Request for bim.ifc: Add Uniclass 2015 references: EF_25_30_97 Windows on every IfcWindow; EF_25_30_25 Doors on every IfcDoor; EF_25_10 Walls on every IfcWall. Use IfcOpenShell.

First a look at what the model holds.

```python
import ifcopenshell

model = ifcopenshell.open("bim.ifc")
print(model.schema)
print("classifications:", [c.Name for c in model.by_type("IfcClassification")])
for ifc_class in ("IfcDoor", "IfcRoof", "IfcStair", "IfcWall", "IfcWindow"):
    print(ifc_class, len(model.by_type(ifc_class)))
```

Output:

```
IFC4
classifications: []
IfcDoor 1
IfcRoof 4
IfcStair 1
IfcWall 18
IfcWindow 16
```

```python
import ifcopenshell
import ifcopenshell.api.classification

model = ifcopenshell.open("bim.ifc")

system = ifcopenshell.api.classification.add_classification(model, classification="Uniclass 2015")

codes = {
    "IfcWindow": ("EF_25_30_97", "Windows"),
    "IfcDoor": ("EF_25_30_25", "Doors"),
    "IfcWall": ("EF_25_10", "Walls"),
}
for ifc_class, (code, name) in codes.items():
    products = model.by_type(ifc_class)
    ifcopenshell.api.classification.add_reference(
        model, products=products, classification=system, identification=code, name=name
    )
    print(code, len(products))

model.write("bim_rev.ifc")
```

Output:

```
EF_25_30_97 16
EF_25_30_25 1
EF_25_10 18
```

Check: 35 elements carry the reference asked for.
